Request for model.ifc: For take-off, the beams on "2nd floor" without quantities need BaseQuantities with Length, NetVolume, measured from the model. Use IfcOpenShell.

First a look at what the model holds.

```python
import ifcopenshell
import ifcopenshell.util.element
import ifcopenshell.util.unit

model = ifcopenshell.open("model.ifc")
print(model.schema)
for unit_type in ("LENGTHUNIT", "AREAUNIT", "VOLUMEUNIT"):
    print(unit_type, ifcopenshell.util.unit.calculate_unit_scale(model, unit_type))
storey = next(s for s in model.by_type("IfcBuildingStorey") if s.Name == "2nd floor")
beams = [e for e in ifcopenshell.util.element.get_decomposition(storey) if e.is_a("IfcBeam")]
for e in sorted(beams, key=lambda e: e.id()):
    print(e.id(), e.is_a(), e.Name, list(ifcopenshell.util.element.get_psets(e, qtos_only=True)), sep=" | ")
```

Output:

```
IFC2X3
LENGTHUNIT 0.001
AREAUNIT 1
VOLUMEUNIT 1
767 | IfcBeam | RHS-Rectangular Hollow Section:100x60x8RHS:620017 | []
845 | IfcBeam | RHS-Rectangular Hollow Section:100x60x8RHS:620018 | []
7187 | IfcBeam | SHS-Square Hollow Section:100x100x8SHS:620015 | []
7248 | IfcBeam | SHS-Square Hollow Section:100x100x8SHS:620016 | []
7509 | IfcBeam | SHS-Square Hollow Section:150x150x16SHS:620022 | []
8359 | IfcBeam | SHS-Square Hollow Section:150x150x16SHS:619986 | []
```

```python
import ifcopenshell
import ifcopenshell.api.pset
import ifcopenshell.geom
import ifcopenshell.util.element
import ifcopenshell.util.shape
import ifcopenshell.util.unit

model = ifcopenshell.open("model.ifc")
unit_scale = ifcopenshell.util.unit.calculate_unit_scale(model)
volume_scale = ifcopenshell.util.unit.calculate_unit_scale(model, "VOLUMEUNIT")
settings = ifcopenshell.geom.settings()

storey = next(s for s in model.by_type("IfcBuildingStorey") if s.Name == "2nd floor")
beams = [e for e in ifcopenshell.util.element.get_decomposition(storey) if e.is_a("IfcBeam")]

for e in sorted(beams, key=lambda e: e.id()):
    if ifcopenshell.util.element.get_psets(e, qtos_only=True, should_inherit=False):
        continue
    # Geometry comes back in metres, in the element's own axes.
    shape = ifcopenshell.geom.create_shape(settings, e)
    values = {
        "Length": ifcopenshell.util.shape.get_max_xyz(shape.geometry) / unit_scale,
        "NetVolume": ifcopenshell.util.shape.get_volume(shape.geometry) / volume_scale,
    }
    qto = ifcopenshell.api.pset.add_qto(model, product=e, name="BaseQuantities")
    ifcopenshell.api.pset.edit_qto(model, qto=qto, properties=values)
    print(e.id(), {k: round(v, 3) for k, v in values.items()})

model.write("model_updated.ifc")
```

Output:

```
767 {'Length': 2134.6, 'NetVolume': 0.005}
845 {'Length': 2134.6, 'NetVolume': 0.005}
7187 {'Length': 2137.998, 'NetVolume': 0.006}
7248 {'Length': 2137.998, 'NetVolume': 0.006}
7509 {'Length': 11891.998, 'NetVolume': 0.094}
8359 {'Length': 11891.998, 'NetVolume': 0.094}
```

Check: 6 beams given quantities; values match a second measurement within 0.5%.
